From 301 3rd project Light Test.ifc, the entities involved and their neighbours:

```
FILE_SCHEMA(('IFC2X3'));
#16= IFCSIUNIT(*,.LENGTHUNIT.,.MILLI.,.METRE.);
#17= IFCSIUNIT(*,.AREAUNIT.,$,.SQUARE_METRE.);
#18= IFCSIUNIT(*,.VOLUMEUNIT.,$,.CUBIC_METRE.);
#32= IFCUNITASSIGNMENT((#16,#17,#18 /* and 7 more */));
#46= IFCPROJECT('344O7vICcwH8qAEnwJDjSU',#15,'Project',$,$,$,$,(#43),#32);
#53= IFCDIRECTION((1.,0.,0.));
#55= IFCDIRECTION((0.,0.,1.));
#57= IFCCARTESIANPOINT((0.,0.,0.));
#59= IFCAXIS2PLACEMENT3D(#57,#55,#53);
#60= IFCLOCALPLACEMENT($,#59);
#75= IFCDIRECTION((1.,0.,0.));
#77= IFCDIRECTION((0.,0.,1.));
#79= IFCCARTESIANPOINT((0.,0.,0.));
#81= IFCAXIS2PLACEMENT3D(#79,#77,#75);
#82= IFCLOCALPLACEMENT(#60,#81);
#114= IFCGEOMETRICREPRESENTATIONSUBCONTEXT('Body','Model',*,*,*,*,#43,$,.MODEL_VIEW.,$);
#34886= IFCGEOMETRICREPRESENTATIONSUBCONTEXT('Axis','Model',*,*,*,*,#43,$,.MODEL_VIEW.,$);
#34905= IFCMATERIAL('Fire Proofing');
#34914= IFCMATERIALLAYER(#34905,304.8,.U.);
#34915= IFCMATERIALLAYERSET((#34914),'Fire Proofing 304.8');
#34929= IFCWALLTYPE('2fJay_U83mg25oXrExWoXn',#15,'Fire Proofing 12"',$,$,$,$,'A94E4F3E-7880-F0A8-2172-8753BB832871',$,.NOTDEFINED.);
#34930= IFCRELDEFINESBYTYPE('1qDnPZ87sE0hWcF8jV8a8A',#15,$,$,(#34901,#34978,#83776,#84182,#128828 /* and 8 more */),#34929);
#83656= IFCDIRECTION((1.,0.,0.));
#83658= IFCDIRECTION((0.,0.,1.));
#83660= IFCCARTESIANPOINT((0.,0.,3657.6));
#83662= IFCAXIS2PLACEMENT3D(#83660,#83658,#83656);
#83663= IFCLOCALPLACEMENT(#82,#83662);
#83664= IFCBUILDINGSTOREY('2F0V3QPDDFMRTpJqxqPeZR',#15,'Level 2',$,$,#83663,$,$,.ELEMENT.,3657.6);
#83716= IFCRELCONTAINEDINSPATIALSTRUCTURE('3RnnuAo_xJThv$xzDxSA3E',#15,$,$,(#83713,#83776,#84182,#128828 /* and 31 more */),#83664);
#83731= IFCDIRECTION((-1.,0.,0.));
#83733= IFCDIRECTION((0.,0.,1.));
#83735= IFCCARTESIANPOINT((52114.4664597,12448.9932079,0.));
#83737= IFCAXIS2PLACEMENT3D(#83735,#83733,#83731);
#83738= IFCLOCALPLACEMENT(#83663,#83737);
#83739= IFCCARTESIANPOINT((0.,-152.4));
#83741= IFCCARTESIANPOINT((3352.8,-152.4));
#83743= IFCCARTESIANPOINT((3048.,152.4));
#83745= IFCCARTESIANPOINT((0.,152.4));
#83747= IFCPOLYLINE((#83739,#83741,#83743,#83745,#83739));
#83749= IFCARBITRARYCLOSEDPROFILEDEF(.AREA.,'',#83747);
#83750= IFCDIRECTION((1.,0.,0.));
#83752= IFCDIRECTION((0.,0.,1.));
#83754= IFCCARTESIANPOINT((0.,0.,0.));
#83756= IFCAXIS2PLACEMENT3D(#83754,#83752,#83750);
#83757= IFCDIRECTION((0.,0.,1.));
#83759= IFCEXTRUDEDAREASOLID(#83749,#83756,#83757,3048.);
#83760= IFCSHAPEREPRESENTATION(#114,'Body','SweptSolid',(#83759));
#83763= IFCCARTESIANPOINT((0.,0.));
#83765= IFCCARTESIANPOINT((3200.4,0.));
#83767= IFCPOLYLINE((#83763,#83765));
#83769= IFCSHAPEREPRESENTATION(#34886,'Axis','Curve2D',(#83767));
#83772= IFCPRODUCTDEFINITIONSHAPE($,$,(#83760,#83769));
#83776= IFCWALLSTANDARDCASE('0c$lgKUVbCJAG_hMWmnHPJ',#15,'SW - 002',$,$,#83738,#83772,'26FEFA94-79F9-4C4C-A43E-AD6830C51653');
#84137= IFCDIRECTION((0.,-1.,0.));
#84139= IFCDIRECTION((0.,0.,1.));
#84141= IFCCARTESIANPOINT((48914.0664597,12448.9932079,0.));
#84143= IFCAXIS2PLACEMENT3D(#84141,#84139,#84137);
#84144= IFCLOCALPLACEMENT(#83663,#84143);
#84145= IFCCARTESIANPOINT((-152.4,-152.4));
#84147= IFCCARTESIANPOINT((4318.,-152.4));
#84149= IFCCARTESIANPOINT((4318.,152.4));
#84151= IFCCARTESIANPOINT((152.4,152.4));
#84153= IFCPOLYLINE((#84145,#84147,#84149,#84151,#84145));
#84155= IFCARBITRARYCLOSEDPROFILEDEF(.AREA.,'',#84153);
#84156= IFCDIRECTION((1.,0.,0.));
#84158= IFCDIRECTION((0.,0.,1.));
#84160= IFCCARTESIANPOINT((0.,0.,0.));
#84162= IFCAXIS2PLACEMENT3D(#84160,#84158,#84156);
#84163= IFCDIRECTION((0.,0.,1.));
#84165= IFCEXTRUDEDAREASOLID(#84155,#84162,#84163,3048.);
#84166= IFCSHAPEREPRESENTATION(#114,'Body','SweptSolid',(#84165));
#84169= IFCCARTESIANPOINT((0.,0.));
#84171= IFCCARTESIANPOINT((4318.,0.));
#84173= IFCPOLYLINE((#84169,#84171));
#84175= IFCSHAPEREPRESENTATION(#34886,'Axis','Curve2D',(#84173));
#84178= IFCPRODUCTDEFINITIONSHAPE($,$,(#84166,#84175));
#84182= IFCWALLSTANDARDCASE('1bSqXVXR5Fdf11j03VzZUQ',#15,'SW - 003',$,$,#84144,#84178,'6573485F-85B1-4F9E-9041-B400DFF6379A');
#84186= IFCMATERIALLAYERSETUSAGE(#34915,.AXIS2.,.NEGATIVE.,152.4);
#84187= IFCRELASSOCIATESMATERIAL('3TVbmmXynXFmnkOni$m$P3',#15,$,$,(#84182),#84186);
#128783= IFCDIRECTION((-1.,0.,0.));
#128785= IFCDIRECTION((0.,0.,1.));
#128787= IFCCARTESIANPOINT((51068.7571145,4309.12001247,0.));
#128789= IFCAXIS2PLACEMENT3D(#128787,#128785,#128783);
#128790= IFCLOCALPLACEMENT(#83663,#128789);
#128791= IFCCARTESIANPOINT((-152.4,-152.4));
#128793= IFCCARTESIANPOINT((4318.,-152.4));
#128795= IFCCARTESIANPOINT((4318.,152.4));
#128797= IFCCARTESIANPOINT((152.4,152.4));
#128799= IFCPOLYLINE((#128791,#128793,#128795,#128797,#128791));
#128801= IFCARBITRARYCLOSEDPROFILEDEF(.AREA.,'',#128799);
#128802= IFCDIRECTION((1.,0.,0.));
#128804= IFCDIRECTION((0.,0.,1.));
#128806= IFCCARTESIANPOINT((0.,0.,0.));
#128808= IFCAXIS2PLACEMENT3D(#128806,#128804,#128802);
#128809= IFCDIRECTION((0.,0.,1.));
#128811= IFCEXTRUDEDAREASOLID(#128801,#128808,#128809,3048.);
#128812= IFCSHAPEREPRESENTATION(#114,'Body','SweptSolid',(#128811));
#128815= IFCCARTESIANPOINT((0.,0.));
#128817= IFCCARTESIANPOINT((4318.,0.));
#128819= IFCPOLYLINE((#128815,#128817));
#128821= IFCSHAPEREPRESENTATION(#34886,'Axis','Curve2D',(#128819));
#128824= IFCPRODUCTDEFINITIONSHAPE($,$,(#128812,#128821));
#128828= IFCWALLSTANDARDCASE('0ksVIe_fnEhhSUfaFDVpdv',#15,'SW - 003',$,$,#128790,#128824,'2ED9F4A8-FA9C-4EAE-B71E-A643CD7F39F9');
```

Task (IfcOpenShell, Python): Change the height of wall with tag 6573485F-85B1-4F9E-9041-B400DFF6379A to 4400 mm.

```python
import ifcopenshell
import ifcopenshell.geom
import ifcopenshell.util.representation
import ifcopenshell.util.shape
import ifcopenshell.util.unit

model = ifcopenshell.open("301 3rd project Light Test.ifc")
unit_scale = ifcopenshell.util.unit.calculate_unit_scale(model)
settings = ifcopenshell.geom.settings()


def volume(element):
    """Net volume in cubic metres, openings subtracted."""
    shape = ifcopenshell.geom.create_shape(settings, element)
    return ifcopenshell.util.shape.get_volume(shape.geometry)


wall = model.by_guid("1bSqXVXR5Fdf11j03VzZUQ")
before = volume(wall)

body = ifcopenshell.util.representation.get_representation(wall, "Model", "Body")
solid = body.Items[0]
old_height = solid.Depth
solid.Depth = 4.4 / unit_scale
after = volume(wall)

print(f"height {old_height:g} -> {solid.Depth:g}, volume {before:.3f} -> {after:.3f} m3")

model.write("301 3rd project Light Test-out.ifc")
```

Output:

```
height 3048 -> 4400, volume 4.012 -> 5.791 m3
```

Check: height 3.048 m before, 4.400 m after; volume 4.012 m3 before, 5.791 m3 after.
